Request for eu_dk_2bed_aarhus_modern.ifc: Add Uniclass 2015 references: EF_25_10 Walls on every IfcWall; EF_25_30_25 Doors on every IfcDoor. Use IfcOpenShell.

First a look at what the model holds.

```python
import ifcopenshell

model = ifcopenshell.open("eu_dk_2bed_aarhus_modern.ifc")
print(model.schema)
print("classifications:", [c.Name for c in model.by_type("IfcClassification")])
for ifc_class in ("IfcDoor", "IfcRoof", "IfcStair", "IfcWall", "IfcWindow"):
    print(ifc_class, len(model.by_type(ifc_class)))
```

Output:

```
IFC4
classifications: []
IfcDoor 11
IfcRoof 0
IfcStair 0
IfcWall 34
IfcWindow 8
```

```python
import ifcopenshell
import ifcopenshell.api.classification

model = ifcopenshell.open("eu_dk_2bed_aarhus_modern.ifc")

system = ifcopenshell.api.classification.add_classification(model, classification="Uniclass 2015")

codes = {
    "IfcWall": ("EF_25_10", "Walls"),
    "IfcDoor": ("EF_25_30_25", "Doors"),
}
for ifc_class, (code, name) in codes.items():
    products = model.by_type(ifc_class)
    ifcopenshell.api.classification.add_reference(
        model, products=products, classification=system, identification=code, name=name
    )
    print(code, len(products))

model.write("eu_dk_2bed_aarhus_modern-out.ifc")
```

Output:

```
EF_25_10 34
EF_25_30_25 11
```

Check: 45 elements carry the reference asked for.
